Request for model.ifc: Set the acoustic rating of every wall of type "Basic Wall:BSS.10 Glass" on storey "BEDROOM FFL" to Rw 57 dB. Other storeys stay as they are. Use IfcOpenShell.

First a look at what the model holds.

```python
import ifcopenshell
import ifcopenshell.util.element

model = ifcopenshell.open("model.ifc")
print(model.schema)
storey = next(s for s in model.by_type("IfcBuildingStorey") if s.Name == "BEDROOM FFL")
walls = [e for e in ifcopenshell.util.element.get_decomposition(storey) if e.is_a("IfcWall")]
seen = {}
for e in walls:
    element_type = ifcopenshell.util.element.get_type(e)
    key = (element_type.Name if element_type != e and element_type else None, ifcopenshell.util.element.get_pset(e, "Pset_WallCommon", "AcousticRating"))
    seen[key] = seen.get(key, 0) + 1
for (name, value), count in sorted(seen.items(), key=str):
    print(count, "x", name, "|", value)
```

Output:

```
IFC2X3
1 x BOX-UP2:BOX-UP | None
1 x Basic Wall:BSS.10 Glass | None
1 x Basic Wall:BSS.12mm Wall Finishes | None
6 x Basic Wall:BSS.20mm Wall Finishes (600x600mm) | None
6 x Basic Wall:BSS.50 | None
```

```python
import ifcopenshell
import ifcopenshell.api.pset
import ifcopenshell.util.element

model = ifcopenshell.open("model.ifc")

storey = next(s for s in model.by_type("IfcBuildingStorey") if s.Name == "BEDROOM FFL")
walls = [e for e in ifcopenshell.util.element.get_decomposition(storey) if e.is_a("IfcWall")]

count = 0
for e in walls:
    element_type = ifcopenshell.util.element.get_type(e)
    if element_type in (None, e) or element_type.Name != "Basic Wall:BSS.10 Glass":
        continue
    # add_pset returns the element's existing set when there is one.
    pset = ifcopenshell.api.pset.add_pset(model, product=e, name="Pset_WallCommon")
    ifcopenshell.api.pset.edit_pset(model, pset=pset, properties={"AcousticRating": "Rw 57 dB"})
    count += 1

print(count, "walls updated")

model.write("model_updated.ifc")
```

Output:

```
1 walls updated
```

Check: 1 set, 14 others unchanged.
